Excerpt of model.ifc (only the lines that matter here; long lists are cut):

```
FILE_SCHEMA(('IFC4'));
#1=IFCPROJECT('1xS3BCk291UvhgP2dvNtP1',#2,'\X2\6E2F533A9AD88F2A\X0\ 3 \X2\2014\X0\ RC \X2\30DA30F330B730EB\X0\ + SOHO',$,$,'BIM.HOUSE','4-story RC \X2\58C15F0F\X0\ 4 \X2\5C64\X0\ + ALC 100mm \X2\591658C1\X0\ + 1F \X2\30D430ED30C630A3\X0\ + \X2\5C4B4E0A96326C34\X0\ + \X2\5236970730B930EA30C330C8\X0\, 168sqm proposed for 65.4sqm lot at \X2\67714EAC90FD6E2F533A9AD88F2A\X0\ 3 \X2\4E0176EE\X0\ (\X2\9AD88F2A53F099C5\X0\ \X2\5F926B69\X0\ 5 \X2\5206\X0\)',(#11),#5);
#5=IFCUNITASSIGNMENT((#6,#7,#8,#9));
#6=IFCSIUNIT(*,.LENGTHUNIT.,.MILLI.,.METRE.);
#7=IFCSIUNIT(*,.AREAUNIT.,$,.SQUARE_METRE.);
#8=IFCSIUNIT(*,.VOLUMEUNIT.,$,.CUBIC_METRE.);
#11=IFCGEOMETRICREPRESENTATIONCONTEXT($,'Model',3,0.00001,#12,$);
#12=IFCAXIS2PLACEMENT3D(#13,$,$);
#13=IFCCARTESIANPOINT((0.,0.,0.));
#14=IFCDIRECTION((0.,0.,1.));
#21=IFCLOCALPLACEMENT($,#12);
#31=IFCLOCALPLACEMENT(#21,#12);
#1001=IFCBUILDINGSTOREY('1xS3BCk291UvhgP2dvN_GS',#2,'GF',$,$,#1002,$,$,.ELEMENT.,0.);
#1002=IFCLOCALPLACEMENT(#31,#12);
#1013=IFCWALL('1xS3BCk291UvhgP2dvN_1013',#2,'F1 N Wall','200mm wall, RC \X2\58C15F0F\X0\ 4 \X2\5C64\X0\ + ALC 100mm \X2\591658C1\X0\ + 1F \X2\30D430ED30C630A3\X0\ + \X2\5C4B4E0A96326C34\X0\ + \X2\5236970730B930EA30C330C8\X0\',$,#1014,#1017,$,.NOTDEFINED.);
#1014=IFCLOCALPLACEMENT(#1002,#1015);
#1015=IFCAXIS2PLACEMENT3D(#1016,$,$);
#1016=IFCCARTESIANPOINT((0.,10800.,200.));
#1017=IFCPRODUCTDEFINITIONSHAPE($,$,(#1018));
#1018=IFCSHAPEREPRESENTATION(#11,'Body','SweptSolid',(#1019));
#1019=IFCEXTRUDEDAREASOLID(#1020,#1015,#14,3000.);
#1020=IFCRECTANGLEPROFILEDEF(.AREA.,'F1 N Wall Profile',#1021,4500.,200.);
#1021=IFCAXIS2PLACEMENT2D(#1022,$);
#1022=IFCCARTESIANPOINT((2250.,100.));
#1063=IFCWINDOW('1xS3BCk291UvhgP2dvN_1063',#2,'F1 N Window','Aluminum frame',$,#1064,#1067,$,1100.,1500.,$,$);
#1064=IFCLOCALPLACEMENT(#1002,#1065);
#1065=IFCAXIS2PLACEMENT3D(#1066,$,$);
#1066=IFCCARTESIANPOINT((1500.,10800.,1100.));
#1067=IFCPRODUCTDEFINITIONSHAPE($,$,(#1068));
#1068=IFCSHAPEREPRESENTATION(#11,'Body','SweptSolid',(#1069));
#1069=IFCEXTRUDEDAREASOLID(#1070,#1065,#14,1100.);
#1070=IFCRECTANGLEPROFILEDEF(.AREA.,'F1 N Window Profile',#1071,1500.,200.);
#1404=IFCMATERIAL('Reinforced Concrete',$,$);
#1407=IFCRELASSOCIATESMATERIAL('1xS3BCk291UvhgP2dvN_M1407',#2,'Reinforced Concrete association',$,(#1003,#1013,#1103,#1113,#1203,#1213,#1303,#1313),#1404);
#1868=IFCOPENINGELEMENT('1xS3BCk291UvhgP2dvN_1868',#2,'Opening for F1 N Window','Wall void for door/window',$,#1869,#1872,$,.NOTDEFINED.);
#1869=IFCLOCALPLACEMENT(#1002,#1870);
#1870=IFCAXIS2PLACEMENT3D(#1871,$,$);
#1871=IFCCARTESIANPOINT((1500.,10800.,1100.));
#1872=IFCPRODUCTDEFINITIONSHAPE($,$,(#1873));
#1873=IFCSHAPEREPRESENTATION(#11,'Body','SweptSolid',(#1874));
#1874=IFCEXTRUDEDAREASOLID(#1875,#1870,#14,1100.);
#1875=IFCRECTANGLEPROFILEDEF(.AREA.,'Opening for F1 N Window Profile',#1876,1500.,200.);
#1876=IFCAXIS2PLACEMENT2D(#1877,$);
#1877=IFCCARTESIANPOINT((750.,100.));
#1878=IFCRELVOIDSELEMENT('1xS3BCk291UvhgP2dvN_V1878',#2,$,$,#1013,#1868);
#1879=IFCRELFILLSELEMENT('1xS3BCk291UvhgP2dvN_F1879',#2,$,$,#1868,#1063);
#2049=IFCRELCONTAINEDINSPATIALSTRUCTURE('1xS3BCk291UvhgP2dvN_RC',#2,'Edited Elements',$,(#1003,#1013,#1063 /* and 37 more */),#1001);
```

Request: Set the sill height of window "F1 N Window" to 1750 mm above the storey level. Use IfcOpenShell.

```python
import numpy as np
import ifcopenshell
import ifcopenshell.api.geometry
import ifcopenshell.geom
import ifcopenshell.util.element
import ifcopenshell.util.placement
import ifcopenshell.util.shape
import ifcopenshell.util.unit

model = ifcopenshell.open("model.ifc")
unit_scale = ifcopenshell.util.unit.calculate_unit_scale(model)

window = model.by_guid("1xS3BCk291UvhgP2dvN_1063")
opening = window.FillsVoids[0].RelatingOpeningElement
storey = ifcopenshell.util.element.get_container(window, ifc_class="IfcBuildingStorey")
level = ifcopenshell.util.placement.get_local_placement(storey.ObjectPlacement)[2, 3]

# The opening's origin need not be at the sill, so measure its lowest point.
shape = ifcopenshell.geom.create_shape(ifcopenshell.geom.settings(), opening)
bottom = ifcopenshell.util.shape.get_shape_bottom_elevation(shape, shape.geometry) / unit_scale
dz = level + 1750.0 - bottom

shift = np.array([0.0, 0.0, dz])
# The window is not placed relative to its opening, so move both.
for product in (opening, window):
    matrix = ifcopenshell.util.placement.get_local_placement(product.ObjectPlacement)
    matrix[:3, 3] += shift
    ifcopenshell.api.geometry.edit_object_placement(model, product=product, matrix=matrix, is_si=False)

print(f"moved by {dz * unit_scale:+.3f} m")

model.write("model_rev.ifc")
```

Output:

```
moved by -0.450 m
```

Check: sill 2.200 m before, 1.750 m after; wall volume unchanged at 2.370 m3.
